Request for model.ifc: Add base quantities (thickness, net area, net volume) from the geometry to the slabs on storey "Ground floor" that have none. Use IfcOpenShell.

First a look at what the model holds.

```python
import ifcopenshell
import ifcopenshell.util.element
import ifcopenshell.util.unit

model = ifcopenshell.open("model.ifc")
print(model.schema)
for unit_type in ("LENGTHUNIT", "AREAUNIT", "VOLUMEUNIT"):
    print(unit_type, ifcopenshell.util.unit.calculate_unit_scale(model, unit_type))
storey = next(s for s in model.by_type("IfcBuildingStorey") if s.Name == "Ground floor")
slabs = [e for e in ifcopenshell.util.element.get_decomposition(storey) if e.is_a("IfcSlab")]
for e in sorted(slabs, key=lambda e: e.id()):
    print(e.id(), e.is_a(), e.Name, list(ifcopenshell.util.element.get_psets(e, qtos_only=True)), sep=" | ")
```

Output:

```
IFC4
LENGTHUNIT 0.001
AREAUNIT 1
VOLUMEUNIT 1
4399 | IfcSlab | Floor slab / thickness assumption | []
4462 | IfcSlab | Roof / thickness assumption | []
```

```python
import ifcopenshell
import ifcopenshell.api.pset
import ifcopenshell.geom
import ifcopenshell.util.element
import ifcopenshell.util.shape
import ifcopenshell.util.unit

model = ifcopenshell.open("model.ifc")
unit_scale = ifcopenshell.util.unit.calculate_unit_scale(model)
area_scale = ifcopenshell.util.unit.calculate_unit_scale(model, "AREAUNIT")
volume_scale = ifcopenshell.util.unit.calculate_unit_scale(model, "VOLUMEUNIT")
settings = ifcopenshell.geom.settings()

storey = next(s for s in model.by_type("IfcBuildingStorey") if s.Name == "Ground floor")
slabs = [e for e in ifcopenshell.util.element.get_decomposition(storey) if e.is_a("IfcSlab")]

for e in sorted(slabs, key=lambda e: e.id()):
    if ifcopenshell.util.element.get_psets(e, qtos_only=True, should_inherit=False):
        continue
    # Geometry comes back in metres, in the element's own axes.
    shape = ifcopenshell.geom.create_shape(settings, e)
    values = {
        "Width": ifcopenshell.util.shape.get_z(shape.geometry) / unit_scale,
        "NetArea": ifcopenshell.util.shape.get_footprint_area(shape.geometry) / area_scale,
        "NetVolume": ifcopenshell.util.shape.get_volume(shape.geometry) / volume_scale,
    }
    qto = ifcopenshell.api.pset.add_qto(model, product=e, name="Qto_SlabBaseQuantities")
    ifcopenshell.api.pset.edit_qto(model, qto=qto, properties=values)
    print(e.id(), {k: round(v, 3) for k, v in values.items()})

model.write("model-out.ifc")
```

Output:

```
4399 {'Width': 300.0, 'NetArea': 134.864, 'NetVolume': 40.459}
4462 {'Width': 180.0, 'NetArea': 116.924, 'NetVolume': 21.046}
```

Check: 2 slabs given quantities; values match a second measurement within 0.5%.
